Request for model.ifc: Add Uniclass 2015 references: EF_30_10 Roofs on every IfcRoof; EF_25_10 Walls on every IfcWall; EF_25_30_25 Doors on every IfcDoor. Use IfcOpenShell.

First a look at what the model holds.

```python
import ifcopenshell

model = ifcopenshell.open("model.ifc")
print(model.schema)
print("classifications:", [c.Name for c in model.by_type("IfcClassification")])
for ifc_class in ("IfcDoor", "IfcRoof", "IfcStair", "IfcWall", "IfcWindow"):
    print(ifc_class, len(model.by_type(ifc_class)))
```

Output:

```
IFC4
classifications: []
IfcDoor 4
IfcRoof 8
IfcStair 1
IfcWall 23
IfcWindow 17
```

```python
import ifcopenshell
import ifcopenshell.api.classification

model = ifcopenshell.open("model.ifc")

system = ifcopenshell.api.classification.add_classification(model, classification="Uniclass 2015")

codes = {
    "IfcRoof": ("EF_30_10", "Roofs"),
    "IfcWall": ("EF_25_10", "Walls"),
    "IfcDoor": ("EF_25_30_25", "Doors"),
}
for ifc_class, (code, name) in codes.items():
    products = model.by_type(ifc_class)
    ifcopenshell.api.classification.add_reference(
        model, products=products, classification=system, identification=code, name=name
    )
    print(code, len(products))

model.write("model_updated.ifc")
```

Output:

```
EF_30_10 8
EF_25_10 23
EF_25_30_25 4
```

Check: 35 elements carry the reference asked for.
